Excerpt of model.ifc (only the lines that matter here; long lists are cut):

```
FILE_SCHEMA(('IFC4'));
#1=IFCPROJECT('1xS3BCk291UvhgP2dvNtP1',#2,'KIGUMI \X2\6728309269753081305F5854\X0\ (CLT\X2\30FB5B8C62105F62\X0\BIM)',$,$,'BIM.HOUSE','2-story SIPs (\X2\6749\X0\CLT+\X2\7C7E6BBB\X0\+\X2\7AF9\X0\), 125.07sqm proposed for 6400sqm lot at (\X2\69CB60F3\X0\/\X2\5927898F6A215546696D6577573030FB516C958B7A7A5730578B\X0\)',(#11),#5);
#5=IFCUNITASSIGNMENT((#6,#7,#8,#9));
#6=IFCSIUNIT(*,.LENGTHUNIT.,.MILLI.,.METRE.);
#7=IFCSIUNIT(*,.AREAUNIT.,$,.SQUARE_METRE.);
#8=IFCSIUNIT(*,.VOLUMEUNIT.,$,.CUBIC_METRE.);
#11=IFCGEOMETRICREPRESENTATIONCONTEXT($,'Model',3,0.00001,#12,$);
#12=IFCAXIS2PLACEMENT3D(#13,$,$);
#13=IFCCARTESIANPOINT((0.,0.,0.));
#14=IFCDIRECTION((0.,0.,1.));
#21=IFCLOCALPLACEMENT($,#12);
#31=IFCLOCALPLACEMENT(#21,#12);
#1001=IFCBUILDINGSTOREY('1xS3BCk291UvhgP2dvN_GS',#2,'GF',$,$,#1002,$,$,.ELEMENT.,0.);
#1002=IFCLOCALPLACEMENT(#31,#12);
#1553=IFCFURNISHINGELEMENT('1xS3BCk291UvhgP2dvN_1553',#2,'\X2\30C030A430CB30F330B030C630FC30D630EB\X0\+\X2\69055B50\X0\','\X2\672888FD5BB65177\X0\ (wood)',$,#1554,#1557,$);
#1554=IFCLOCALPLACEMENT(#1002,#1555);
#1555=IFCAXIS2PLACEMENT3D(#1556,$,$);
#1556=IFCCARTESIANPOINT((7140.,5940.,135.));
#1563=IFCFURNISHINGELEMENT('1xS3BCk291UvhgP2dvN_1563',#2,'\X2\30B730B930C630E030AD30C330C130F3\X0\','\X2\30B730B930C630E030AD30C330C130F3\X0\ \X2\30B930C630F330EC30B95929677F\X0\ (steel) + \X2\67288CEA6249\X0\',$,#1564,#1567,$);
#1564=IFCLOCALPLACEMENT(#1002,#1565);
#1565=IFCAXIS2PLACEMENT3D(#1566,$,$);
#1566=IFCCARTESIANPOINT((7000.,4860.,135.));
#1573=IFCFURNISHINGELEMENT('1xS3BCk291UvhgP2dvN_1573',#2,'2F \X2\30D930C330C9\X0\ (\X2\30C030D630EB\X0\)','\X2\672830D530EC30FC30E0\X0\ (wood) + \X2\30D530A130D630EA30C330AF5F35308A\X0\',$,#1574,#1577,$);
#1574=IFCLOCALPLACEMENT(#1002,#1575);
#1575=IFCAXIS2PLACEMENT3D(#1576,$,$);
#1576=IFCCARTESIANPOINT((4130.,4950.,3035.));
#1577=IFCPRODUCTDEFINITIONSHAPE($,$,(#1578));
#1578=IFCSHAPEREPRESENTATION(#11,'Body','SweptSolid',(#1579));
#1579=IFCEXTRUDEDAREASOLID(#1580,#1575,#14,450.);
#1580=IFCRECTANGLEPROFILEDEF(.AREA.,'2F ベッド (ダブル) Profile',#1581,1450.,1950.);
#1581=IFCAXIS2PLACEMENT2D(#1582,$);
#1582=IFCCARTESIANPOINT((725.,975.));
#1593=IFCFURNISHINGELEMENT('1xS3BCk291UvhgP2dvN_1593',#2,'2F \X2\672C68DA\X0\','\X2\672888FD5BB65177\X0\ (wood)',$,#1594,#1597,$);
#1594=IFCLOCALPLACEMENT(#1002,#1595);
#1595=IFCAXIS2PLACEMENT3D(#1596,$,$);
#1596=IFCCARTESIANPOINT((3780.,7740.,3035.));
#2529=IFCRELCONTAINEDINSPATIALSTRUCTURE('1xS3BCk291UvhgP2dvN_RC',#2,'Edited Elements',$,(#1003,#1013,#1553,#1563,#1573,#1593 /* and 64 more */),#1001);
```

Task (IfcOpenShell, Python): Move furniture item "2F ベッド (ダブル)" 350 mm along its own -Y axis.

```python
import ifcopenshell
import ifcopenshell.api.geometry
import ifcopenshell.util.placement
import ifcopenshell.util.unit

model = ifcopenshell.open("model.ifc")
unit_scale = ifcopenshell.util.unit.calculate_unit_scale(model)

item = model.by_guid("1xS3BCk291UvhgP2dvN_1573")
matrix = ifcopenshell.util.placement.get_local_placement(item.ObjectPlacement)
matrix[:3, 3] -= matrix[:3, 1] * 0.35 / unit_scale
ifcopenshell.api.geometry.edit_object_placement(model, product=item, matrix=matrix, is_si=False)

print(ifcopenshell.util.placement.get_local_placement(item.ObjectPlacement).round(3) + 0.0)

model.write("model_edited.ifc")
```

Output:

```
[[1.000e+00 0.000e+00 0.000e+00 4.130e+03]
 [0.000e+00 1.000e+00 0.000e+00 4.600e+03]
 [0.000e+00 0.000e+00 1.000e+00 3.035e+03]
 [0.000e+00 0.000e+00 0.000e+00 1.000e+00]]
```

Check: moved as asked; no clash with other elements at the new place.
